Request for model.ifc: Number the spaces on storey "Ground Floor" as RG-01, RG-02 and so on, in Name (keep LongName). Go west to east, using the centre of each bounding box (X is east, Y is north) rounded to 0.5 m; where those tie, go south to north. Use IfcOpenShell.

First a look at what the model holds.

```python
import ifcopenshell
import ifcopenshell.util.element
import ifcopenshell.util.placement

model = ifcopenshell.open("model.ifc")
print(model.schema)
storey = next(s for s in model.by_type("IfcBuildingStorey") if s.Name == "Ground Floor")
spaces = [e for e in ifcopenshell.util.element.get_decomposition(storey) if e.is_a("IfcSpace")]
for e in sorted(spaces, key=lambda e: e.id()):
    origin = ifcopenshell.util.placement.get_local_placement(e.ObjectPlacement)[:3, 3]
    print(e.id(), e.Name, e.LongName, origin.round(2) + 0.0, sep=" | ")
```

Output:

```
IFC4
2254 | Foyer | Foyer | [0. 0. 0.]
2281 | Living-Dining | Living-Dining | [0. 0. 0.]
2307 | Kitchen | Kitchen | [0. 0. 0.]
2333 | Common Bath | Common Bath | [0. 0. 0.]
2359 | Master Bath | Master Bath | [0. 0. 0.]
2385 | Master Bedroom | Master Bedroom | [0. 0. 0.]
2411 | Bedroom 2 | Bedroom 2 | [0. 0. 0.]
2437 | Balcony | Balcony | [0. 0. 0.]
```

```python
import ifcopenshell
import ifcopenshell.geom
import ifcopenshell.util.element
import ifcopenshell.util.shape

model = ifcopenshell.open("model.ifc")
settings = ifcopenshell.geom.settings()
settings.set("use-world-coords", True)


def centre(element):
    shape = ifcopenshell.geom.create_shape(settings, element)
    return ifcopenshell.util.shape.get_bbox_centroid(shape.geometry)


storey = next(s for s in model.by_type("IfcBuildingStorey") if s.Name == "Ground Floor")
spaces = [e for e in ifcopenshell.util.element.get_decomposition(storey) if e.is_a("IfcSpace")]

# Insertion points can sit at a corner or the storey origin, so sort by the geometry (in metres).
centres = {e: centre(e) for e in spaces}
spaces.sort(key=lambda e: (round(centres[e][0] / 0.5), centres[e][1]))

for i, e in enumerate(spaces, start=1):
    number = f"RG-{i:02d}"
    e.Name = number
    print(e.id(), number)

model.write("model-out.ifc")
```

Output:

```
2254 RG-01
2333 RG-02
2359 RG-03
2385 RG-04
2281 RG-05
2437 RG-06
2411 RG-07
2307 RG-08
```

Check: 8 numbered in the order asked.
